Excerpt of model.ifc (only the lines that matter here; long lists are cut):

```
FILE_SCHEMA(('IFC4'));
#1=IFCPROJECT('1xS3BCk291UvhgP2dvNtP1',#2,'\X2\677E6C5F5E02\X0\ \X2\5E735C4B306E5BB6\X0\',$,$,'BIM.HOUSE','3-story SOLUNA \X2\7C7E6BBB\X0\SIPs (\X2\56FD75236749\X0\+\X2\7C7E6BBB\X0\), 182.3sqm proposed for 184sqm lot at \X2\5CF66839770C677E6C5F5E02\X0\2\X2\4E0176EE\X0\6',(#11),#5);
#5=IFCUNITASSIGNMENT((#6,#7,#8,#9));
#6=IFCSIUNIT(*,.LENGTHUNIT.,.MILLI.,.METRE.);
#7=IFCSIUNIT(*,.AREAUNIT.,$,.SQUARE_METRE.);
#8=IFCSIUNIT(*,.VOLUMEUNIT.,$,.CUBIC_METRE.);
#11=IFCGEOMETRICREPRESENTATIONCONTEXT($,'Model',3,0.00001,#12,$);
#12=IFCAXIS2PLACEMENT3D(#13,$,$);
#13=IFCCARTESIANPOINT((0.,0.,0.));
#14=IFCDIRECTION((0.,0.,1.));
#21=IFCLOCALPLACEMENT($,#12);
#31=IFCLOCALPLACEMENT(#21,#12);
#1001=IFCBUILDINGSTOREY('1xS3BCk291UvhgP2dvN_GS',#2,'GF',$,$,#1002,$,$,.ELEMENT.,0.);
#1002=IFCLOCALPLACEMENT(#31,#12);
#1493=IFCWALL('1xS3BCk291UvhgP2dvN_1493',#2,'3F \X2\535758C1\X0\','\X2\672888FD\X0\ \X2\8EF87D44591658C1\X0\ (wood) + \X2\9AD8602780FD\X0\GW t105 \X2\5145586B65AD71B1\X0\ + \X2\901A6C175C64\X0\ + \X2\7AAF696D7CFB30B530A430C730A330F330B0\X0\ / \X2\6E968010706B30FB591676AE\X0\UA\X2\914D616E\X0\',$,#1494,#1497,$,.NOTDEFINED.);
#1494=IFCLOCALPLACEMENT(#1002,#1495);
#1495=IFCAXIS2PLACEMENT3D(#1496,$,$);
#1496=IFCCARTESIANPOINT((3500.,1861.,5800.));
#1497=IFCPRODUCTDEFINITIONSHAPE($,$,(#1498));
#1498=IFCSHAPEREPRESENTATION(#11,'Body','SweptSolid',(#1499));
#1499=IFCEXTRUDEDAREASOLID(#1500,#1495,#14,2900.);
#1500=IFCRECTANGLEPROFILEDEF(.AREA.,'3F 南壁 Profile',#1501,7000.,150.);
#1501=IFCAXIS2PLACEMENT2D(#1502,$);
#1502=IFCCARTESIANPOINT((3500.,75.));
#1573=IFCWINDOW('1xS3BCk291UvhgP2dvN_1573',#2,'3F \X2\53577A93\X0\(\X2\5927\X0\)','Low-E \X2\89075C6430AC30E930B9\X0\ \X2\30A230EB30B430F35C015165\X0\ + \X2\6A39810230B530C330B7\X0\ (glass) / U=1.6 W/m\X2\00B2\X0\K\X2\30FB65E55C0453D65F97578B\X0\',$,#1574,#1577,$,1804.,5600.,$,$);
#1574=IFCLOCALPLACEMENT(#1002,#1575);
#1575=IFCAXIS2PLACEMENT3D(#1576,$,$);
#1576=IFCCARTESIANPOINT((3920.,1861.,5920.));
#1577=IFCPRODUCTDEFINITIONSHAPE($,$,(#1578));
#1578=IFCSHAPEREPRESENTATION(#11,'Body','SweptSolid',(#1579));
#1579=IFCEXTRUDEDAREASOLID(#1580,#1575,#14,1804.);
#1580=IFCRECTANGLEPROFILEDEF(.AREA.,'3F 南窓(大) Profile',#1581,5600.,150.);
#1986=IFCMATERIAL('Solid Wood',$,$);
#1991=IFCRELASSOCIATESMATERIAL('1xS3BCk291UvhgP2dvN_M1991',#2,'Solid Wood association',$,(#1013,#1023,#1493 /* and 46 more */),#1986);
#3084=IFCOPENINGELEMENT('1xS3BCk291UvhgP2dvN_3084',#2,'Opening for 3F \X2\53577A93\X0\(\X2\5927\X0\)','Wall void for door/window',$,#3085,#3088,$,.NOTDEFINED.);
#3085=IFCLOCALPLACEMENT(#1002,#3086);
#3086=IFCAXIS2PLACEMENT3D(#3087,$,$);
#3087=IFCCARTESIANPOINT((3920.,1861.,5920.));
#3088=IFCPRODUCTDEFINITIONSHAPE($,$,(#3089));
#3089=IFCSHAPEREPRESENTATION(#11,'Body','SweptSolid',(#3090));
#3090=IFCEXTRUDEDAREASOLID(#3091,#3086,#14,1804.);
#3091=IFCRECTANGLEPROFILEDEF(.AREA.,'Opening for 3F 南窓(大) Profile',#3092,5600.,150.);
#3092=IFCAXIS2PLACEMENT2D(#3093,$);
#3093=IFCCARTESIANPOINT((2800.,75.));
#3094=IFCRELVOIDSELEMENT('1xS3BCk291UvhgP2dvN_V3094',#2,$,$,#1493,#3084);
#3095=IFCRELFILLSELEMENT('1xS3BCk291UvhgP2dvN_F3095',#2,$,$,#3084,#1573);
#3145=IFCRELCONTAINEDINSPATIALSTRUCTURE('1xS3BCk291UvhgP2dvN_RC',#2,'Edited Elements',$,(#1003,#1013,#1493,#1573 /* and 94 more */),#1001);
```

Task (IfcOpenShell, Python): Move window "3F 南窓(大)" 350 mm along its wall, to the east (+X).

```python
import ifcopenshell
import ifcopenshell.api.geometry
import ifcopenshell.util.placement

model = ifcopenshell.open("model.ifc")

window = model.by_guid("1xS3BCk291UvhgP2dvN_1573")
opening = window.FillsVoids[0].RelatingOpeningElement
wall = opening.VoidsElements[0].RelatingBuildingElement

wall_matrix = ifcopenshell.util.placement.get_local_placement(wall.ObjectPlacement)
shift = wall_matrix[:3, 0] * 350.0
before = ifcopenshell.util.placement.get_local_placement(window.ObjectPlacement)[:3, 3].copy()

# The window is not placed relative to its opening, so move both.
for product in (opening, window):
    matrix = ifcopenshell.util.placement.get_local_placement(product.ObjectPlacement)
    matrix[:3, 3] += shift
    ifcopenshell.api.geometry.edit_object_placement(model, product=product, matrix=matrix, is_si=False)

after = ifcopenshell.util.placement.get_local_placement(window.ObjectPlacement)[:3, 3]
print("window moved by", (after - before).round(3) + 0.0)

model.write("model_v2.ifc")
```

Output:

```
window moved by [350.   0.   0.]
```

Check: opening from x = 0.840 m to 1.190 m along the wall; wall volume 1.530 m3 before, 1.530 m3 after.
